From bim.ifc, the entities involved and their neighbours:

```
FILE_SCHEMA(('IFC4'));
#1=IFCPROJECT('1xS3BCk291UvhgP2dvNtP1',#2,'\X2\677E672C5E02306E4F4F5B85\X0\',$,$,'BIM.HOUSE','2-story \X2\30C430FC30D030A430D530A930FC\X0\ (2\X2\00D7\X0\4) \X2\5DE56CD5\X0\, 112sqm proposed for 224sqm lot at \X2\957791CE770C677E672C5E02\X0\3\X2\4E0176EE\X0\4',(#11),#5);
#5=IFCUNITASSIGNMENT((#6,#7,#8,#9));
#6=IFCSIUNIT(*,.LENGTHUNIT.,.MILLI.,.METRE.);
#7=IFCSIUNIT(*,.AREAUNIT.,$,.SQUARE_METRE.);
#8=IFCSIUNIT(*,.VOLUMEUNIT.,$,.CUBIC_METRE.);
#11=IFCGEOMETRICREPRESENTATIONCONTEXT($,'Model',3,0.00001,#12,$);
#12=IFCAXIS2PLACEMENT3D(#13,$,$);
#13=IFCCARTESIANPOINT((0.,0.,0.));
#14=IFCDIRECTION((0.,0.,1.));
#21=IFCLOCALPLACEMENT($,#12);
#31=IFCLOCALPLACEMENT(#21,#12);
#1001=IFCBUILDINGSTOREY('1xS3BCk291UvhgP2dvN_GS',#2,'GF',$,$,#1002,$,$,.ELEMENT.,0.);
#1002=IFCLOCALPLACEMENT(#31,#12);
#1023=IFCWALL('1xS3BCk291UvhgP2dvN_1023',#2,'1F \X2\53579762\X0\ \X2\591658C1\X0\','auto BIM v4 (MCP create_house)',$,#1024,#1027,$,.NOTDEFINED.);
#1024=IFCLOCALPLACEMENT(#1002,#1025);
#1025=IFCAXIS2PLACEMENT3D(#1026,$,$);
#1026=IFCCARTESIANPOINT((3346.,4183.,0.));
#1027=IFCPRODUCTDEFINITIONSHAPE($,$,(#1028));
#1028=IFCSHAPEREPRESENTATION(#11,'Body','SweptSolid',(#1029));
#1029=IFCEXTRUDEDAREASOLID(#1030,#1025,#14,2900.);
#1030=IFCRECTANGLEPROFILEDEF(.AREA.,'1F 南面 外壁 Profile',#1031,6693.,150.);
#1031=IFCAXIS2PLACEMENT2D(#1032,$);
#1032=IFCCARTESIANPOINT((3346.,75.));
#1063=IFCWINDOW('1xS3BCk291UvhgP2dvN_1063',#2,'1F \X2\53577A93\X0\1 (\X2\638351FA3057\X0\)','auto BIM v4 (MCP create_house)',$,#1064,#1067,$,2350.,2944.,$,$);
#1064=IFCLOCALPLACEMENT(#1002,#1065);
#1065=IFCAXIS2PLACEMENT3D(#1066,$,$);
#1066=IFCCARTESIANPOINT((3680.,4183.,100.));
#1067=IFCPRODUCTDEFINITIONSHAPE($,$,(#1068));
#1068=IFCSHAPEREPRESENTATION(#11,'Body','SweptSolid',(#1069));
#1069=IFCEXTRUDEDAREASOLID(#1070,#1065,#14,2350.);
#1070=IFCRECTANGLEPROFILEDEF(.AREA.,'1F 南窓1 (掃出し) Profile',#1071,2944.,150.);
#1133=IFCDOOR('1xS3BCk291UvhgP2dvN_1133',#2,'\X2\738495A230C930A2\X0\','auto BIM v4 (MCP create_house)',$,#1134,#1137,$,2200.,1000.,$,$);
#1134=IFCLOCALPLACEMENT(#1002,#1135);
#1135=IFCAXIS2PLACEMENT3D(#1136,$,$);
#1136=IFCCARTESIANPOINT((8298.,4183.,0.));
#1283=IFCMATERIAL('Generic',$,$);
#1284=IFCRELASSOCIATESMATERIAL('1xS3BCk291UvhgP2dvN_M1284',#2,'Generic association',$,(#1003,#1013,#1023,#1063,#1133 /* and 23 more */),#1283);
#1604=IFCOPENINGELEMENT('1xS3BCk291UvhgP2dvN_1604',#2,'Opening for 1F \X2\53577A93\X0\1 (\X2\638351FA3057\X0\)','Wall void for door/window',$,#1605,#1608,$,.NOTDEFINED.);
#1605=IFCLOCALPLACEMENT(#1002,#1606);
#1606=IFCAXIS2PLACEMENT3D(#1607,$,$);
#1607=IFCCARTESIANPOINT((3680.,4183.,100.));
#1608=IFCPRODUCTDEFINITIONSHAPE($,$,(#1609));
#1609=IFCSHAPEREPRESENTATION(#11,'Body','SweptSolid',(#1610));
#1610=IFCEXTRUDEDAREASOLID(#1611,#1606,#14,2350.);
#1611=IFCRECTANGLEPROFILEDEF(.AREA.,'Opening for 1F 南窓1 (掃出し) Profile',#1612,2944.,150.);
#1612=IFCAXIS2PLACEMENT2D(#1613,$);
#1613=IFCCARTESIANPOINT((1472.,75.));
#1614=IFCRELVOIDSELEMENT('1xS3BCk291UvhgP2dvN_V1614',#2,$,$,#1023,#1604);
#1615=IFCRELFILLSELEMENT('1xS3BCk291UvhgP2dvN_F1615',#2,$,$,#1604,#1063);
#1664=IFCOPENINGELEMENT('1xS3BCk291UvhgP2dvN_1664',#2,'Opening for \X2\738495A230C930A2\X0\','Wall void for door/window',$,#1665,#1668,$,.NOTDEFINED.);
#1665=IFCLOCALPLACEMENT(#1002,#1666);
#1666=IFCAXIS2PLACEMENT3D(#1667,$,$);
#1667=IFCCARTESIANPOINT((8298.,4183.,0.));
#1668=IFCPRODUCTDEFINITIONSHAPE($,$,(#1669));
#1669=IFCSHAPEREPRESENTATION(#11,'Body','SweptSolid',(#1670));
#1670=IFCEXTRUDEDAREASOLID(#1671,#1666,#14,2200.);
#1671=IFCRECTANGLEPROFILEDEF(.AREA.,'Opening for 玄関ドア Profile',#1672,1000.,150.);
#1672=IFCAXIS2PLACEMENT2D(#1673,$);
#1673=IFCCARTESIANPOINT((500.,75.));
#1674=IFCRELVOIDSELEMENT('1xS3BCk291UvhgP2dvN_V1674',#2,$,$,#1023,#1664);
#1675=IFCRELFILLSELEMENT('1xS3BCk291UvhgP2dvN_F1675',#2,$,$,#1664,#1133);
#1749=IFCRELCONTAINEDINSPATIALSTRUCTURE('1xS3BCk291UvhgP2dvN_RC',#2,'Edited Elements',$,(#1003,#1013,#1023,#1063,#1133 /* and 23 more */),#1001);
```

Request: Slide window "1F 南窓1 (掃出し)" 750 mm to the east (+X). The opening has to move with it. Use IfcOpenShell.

```python
import ifcopenshell
import ifcopenshell.api.geometry
import ifcopenshell.util.placement
import ifcopenshell.util.unit

model = ifcopenshell.open("bim.ifc")
unit_scale = ifcopenshell.util.unit.calculate_unit_scale(model)

window = model.by_guid("1xS3BCk291UvhgP2dvN_1063")
opening = window.FillsVoids[0].RelatingOpeningElement
wall = opening.VoidsElements[0].RelatingBuildingElement

wall_matrix = ifcopenshell.util.placement.get_local_placement(wall.ObjectPlacement)
shift = wall_matrix[:3, 0] * 0.75 / unit_scale
before = ifcopenshell.util.placement.get_local_placement(window.ObjectPlacement)[:3, 3].copy()

# The window is not placed relative to its opening, so move both.
for product in (opening, window):
    matrix = ifcopenshell.util.placement.get_local_placement(product.ObjectPlacement)
    matrix[:3, 3] += shift
    ifcopenshell.api.geometry.edit_object_placement(model, product=product, matrix=matrix, is_si=False)

after = ifcopenshell.util.placement.get_local_placement(window.ObjectPlacement)[:3, 3]
print("window moved by", (after - before).round(3) + 0.0)

model.write("bim_rev.ifc")
```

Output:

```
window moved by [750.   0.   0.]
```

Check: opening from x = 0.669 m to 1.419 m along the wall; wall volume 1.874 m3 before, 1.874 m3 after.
